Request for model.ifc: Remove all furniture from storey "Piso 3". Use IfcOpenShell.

First a look at what the model holds.

```python
import ifcopenshell
import ifcopenshell.util.element

model = ifcopenshell.open("model.ifc")
print(model.schema)
storey = next(s for s in model.by_type("IfcBuildingStorey") if s.Name == "Piso 3")
furniture = [e for e in ifcopenshell.util.element.get_decomposition(storey) if e.is_a("IfcFurnishingElement")]
seen = {}
for e in furniture:
    element_type = ifcopenshell.util.element.get_type(e)
    name = element_type.Name if element_type not in (None, e) else None
    seen[name] = seen.get(name, 0) + 1
for name, count in sorted(seen.items(), key=str):
    print(count, "x", name)
```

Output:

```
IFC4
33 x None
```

```python
import ifcopenshell
import ifcopenshell.api.root
import ifcopenshell.util.element

model = ifcopenshell.open("model.ifc")

storey = next(s for s in model.by_type("IfcBuildingStorey") if s.Name == "Piso 3")
furniture = [e for e in ifcopenshell.util.element.get_decomposition(storey) if e.is_a("IfcFurnishingElement")]

for e in furniture:
    ifcopenshell.api.root.remove_product(model, product=e)
print(len(furniture), "removed")

model.write("model_edited.ifc")
```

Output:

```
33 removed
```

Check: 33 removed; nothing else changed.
